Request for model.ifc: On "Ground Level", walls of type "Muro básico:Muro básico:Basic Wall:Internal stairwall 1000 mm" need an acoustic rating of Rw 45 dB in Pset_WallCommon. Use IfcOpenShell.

First a look at what the model holds.

```python
import ifcopenshell
import ifcopenshell.util.element

model = ifcopenshell.open("model.ifc")
print(model.schema)
storey = next(s for s in model.by_type("IfcBuildingStorey") if s.Name == "Ground Level")
walls = [e for e in ifcopenshell.util.element.get_decomposition(storey) if e.is_a("IfcWall")]
seen = {}
for e in walls:
    element_type = ifcopenshell.util.element.get_type(e)
    key = (element_type.Name if element_type != e and element_type else None, ifcopenshell.util.element.get_pset(e, "Pset_WallCommon", "AcousticRating"))
    seen[key] = seen.get(key, 0) + 1
for (name, value), count in sorted(seen.items(), key=str):
    print(count, "x", name, "|", value)
```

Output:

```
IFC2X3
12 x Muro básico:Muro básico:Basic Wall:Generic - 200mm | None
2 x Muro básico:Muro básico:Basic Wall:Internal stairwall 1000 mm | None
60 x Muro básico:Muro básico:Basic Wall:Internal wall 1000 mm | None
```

```python
import ifcopenshell
import ifcopenshell.api.pset
import ifcopenshell.util.element

model = ifcopenshell.open("model.ifc")

storey = next(s for s in model.by_type("IfcBuildingStorey") if s.Name == "Ground Level")
walls = [e for e in ifcopenshell.util.element.get_decomposition(storey) if e.is_a("IfcWall")]

count = 0
for e in walls:
    element_type = ifcopenshell.util.element.get_type(e)
    if element_type in (None, e) or element_type.Name != "Muro básico:Muro básico:Basic Wall:Internal stairwall 1000 mm":
        continue
    # add_pset returns the element's existing set when there is one.
    pset = ifcopenshell.api.pset.add_pset(model, product=e, name="Pset_WallCommon")
    ifcopenshell.api.pset.edit_pset(model, pset=pset, properties={"AcousticRating": "Rw 45 dB"})
    count += 1

print(count, "walls updated")

model.write("model_rev.ifc")
```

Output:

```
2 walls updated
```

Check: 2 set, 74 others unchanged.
